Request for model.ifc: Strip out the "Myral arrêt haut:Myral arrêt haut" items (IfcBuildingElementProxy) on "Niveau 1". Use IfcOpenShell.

First a look at what the model holds.

```python
import ifcopenshell
import ifcopenshell.util.element

model = ifcopenshell.open("model.ifc")
print(model.schema)
storey = next(s for s in model.by_type("IfcBuildingStorey") if s.Name == "Niveau 1")
proxies = [e for e in ifcopenshell.util.element.get_decomposition(storey) if e.is_a("IfcBuildingElementProxy")]
seen = {}
for e in proxies:
    element_type = ifcopenshell.util.element.get_type(e)
    name = element_type.Name if element_type not in (None, e) else None
    seen[name] = seen.get(name, 0) + 1
for name, count in sorted(seen.items(), key=str):
    print(count, "x", name)
```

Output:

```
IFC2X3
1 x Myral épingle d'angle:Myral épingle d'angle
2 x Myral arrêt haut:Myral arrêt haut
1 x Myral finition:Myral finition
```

```python
import ifcopenshell
import ifcopenshell.api.root
import ifcopenshell.util.element

model = ifcopenshell.open("model.ifc")

storey = next(s for s in model.by_type("IfcBuildingStorey") if s.Name == "Niveau 1")
proxies = [e for e in ifcopenshell.util.element.get_decomposition(storey) if e.is_a("IfcBuildingElementProxy")]
targets = [e for e in proxies if (t := ifcopenshell.util.element.get_type(e)) not in (None, e) and t.Name == "Myral arrêt haut:Myral arrêt haut"]

for e in targets:
    ifcopenshell.api.root.remove_product(model, product=e)
print(len(targets), "removed")

model.write("model_edited.ifc")
```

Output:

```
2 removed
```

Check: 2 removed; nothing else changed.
